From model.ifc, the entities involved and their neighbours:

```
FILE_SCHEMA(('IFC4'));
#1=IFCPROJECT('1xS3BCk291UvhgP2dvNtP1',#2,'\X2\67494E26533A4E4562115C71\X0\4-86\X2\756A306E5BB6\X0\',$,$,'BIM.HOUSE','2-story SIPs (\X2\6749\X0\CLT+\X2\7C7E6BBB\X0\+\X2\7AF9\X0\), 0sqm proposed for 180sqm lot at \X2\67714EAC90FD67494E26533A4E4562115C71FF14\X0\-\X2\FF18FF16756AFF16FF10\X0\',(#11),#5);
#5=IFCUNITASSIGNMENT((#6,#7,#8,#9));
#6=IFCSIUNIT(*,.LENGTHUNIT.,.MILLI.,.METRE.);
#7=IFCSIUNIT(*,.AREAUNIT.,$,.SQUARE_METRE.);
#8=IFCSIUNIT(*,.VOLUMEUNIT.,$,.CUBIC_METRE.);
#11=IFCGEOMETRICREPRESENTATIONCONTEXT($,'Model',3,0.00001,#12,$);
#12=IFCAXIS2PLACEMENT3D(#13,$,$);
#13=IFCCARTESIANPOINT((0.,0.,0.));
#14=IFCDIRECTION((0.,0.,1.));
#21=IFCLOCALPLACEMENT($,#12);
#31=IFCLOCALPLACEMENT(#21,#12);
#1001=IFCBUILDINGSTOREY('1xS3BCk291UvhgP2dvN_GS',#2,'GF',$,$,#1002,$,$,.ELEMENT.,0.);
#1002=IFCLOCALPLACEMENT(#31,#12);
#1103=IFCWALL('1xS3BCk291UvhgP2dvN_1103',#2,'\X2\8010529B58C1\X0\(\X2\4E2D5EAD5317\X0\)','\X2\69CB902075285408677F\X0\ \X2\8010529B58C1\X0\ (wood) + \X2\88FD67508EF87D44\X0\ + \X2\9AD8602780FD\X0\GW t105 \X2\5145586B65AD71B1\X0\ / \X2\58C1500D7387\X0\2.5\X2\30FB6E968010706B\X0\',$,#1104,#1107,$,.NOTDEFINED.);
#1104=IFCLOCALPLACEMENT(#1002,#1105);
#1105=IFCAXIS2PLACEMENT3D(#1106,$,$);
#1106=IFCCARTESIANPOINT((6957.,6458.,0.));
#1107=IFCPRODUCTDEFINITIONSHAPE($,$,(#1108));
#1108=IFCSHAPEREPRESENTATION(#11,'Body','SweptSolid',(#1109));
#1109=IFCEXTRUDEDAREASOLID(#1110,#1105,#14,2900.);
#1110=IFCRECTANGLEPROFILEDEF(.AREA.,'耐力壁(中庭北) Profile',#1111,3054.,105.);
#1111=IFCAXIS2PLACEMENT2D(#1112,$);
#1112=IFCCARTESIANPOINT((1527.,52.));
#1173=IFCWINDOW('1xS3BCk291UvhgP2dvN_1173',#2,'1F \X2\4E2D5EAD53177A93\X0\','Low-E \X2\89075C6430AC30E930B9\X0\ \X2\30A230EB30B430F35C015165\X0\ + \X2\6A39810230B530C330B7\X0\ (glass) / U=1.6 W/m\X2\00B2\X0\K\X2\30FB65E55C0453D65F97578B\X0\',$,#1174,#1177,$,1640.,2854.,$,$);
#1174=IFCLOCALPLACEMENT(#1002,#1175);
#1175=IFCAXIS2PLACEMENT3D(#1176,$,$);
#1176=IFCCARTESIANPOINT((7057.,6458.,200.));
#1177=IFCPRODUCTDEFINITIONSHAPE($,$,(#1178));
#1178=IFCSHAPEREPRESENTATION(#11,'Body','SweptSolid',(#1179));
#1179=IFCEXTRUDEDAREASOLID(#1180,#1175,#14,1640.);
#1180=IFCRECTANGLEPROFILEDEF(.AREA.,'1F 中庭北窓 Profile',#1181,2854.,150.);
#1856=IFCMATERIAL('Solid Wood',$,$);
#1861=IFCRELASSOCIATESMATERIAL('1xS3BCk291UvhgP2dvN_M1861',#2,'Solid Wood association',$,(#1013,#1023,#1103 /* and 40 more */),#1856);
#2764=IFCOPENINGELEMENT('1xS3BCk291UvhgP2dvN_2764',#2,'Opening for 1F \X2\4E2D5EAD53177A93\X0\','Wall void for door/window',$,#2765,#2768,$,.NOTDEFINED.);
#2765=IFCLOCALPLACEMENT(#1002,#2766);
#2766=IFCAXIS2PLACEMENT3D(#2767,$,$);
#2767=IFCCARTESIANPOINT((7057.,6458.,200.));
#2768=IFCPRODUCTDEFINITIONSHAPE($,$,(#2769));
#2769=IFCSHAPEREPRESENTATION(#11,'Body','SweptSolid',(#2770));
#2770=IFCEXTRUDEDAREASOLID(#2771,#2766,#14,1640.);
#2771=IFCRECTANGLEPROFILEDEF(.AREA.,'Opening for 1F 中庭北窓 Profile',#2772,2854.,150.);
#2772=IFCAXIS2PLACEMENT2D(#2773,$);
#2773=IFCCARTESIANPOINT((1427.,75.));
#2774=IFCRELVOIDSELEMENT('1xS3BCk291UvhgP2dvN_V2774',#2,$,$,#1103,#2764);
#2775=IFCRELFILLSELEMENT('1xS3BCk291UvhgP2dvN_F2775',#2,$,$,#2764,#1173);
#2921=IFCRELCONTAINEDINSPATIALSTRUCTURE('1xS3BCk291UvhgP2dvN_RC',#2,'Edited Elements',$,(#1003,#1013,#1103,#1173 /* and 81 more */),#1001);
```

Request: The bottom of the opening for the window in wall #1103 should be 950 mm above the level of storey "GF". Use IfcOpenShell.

```python
import numpy as np
import ifcopenshell
import ifcopenshell.api.geometry
import ifcopenshell.geom
import ifcopenshell.util.element
import ifcopenshell.util.placement
import ifcopenshell.util.shape
import ifcopenshell.util.unit

model = ifcopenshell.open("model.ifc")
unit_scale = ifcopenshell.util.unit.calculate_unit_scale(model)

window = model.by_guid("1xS3BCk291UvhgP2dvN_1173")
opening = window.FillsVoids[0].RelatingOpeningElement
storey = ifcopenshell.util.element.get_container(window, ifc_class="IfcBuildingStorey")
level = ifcopenshell.util.placement.get_local_placement(storey.ObjectPlacement)[2, 3]

# The opening's origin need not be at the sill, so measure its lowest point.
shape = ifcopenshell.geom.create_shape(ifcopenshell.geom.settings(), opening)
bottom = ifcopenshell.util.shape.get_shape_bottom_elevation(shape, shape.geometry) / unit_scale
dz = level + 950.0 - bottom

shift = np.array([0.0, 0.0, dz])
# The window is not placed relative to its opening, so move both.
for product in (opening, window):
    matrix = ifcopenshell.util.placement.get_local_placement(product.ObjectPlacement)
    matrix[:3, 3] += shift
    ifcopenshell.api.geometry.edit_object_placement(model, product=product, matrix=matrix, is_si=False)

print(f"moved by {dz * unit_scale:+.3f} m")

model.write("model_rev.ifc")
```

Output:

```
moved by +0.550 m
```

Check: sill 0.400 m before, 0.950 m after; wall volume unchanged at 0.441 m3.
